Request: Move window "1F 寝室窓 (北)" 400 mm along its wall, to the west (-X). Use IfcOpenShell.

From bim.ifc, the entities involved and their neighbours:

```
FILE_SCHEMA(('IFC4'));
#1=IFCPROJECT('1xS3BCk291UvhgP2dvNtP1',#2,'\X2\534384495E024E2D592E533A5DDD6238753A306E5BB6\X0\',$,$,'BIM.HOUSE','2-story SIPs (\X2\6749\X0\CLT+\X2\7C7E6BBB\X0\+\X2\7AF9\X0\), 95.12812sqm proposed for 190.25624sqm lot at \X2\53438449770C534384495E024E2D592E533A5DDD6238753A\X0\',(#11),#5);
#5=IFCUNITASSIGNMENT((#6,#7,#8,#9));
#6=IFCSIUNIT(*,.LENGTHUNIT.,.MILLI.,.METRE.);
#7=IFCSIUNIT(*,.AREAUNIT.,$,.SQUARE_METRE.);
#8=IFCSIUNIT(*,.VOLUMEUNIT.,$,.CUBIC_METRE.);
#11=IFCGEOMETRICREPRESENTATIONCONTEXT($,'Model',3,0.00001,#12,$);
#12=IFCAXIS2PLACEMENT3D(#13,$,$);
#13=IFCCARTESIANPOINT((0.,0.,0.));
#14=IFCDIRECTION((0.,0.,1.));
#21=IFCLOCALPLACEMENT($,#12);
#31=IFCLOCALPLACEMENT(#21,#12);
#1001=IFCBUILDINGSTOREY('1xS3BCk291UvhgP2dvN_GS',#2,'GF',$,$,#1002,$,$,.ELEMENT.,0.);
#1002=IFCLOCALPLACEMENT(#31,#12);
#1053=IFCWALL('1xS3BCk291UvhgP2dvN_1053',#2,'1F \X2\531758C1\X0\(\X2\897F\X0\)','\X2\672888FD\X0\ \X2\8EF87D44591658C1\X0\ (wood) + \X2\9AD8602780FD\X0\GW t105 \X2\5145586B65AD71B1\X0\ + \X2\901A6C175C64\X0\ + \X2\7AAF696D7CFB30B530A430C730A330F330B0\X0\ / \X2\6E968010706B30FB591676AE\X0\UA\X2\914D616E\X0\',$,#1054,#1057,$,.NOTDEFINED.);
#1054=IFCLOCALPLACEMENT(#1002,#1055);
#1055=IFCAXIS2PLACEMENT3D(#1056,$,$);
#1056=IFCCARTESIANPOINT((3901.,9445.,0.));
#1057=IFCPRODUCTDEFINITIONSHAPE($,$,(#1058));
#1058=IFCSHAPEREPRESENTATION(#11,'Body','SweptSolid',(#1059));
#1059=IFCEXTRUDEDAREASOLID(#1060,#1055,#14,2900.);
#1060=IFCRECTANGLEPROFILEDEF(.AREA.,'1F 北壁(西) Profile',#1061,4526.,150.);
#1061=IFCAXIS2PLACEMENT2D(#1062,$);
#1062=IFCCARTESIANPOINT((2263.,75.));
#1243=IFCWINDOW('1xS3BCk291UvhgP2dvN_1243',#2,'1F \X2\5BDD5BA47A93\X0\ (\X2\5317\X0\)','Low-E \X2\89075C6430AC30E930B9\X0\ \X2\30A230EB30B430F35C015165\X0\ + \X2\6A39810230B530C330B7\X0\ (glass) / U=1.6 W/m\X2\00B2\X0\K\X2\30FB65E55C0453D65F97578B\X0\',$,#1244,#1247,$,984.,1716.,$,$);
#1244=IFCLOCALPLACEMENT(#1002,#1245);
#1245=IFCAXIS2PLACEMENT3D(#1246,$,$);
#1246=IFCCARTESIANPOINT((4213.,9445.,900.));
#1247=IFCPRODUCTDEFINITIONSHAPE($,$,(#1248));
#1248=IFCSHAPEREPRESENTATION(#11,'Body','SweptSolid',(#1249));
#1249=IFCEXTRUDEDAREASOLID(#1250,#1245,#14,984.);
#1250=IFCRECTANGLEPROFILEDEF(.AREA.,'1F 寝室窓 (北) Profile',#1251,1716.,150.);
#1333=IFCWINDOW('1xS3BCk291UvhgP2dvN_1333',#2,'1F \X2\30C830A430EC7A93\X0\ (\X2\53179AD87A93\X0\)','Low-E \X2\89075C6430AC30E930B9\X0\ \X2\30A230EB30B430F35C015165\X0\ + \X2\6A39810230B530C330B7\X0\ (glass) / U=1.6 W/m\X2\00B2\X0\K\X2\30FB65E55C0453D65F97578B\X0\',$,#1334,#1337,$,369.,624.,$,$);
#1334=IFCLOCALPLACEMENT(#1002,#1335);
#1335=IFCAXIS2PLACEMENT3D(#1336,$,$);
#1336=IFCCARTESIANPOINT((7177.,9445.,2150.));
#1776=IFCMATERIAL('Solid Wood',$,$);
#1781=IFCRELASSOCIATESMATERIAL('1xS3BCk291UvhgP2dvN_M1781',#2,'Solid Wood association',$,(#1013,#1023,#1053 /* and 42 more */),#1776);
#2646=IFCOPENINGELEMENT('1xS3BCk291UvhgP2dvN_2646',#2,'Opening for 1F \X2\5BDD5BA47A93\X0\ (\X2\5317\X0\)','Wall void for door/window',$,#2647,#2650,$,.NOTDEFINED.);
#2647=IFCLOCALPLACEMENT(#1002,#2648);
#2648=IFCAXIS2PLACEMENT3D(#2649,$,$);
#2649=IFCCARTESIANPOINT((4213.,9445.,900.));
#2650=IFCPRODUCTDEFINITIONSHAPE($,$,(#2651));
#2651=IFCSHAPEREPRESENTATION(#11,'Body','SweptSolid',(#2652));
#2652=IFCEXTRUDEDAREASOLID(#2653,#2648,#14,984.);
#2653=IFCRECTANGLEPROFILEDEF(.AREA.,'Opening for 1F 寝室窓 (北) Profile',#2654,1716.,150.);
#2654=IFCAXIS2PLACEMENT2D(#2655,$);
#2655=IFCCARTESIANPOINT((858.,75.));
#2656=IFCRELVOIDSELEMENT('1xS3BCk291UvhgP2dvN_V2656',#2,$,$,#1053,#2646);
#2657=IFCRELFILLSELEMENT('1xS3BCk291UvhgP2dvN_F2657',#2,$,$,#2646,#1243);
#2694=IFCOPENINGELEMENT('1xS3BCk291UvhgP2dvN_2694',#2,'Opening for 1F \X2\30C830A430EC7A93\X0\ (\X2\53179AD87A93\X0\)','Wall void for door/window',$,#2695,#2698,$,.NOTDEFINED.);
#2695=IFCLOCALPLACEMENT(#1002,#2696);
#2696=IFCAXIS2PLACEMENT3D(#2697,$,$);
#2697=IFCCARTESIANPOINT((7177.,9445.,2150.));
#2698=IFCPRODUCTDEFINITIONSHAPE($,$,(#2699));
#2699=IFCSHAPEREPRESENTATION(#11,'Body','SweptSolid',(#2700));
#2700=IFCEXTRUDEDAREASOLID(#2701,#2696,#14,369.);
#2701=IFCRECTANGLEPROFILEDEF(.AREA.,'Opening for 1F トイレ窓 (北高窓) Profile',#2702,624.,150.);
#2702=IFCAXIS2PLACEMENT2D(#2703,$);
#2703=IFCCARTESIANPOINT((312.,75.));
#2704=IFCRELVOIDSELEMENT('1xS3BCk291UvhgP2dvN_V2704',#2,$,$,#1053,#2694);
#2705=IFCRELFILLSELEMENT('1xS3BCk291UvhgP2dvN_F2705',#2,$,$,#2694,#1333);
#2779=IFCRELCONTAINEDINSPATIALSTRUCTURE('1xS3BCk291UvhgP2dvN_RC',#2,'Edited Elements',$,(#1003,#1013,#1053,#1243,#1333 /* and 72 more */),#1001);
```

```python
import ifcopenshell
import ifcopenshell.api.geometry
import ifcopenshell.util.placement
import ifcopenshell.util.unit

model = ifcopenshell.open("bim.ifc")
unit_scale = ifcopenshell.util.unit.calculate_unit_scale(model)

window = model.by_id(1243)
opening = window.FillsVoids[0].RelatingOpeningElement
wall = opening.VoidsElements[0].RelatingBuildingElement

wall_matrix = ifcopenshell.util.placement.get_local_placement(wall.ObjectPlacement)
shift = wall_matrix[:3, 0] * -0.4 / unit_scale
before = ifcopenshell.util.placement.get_local_placement(window.ObjectPlacement)[:3, 3].copy()

# The window is not placed relative to its opening, so move both.
for product in (opening, window):
    matrix = ifcopenshell.util.placement.get_local_placement(product.ObjectPlacement)
    matrix[:3, 3] += shift
    ifcopenshell.api.geometry.edit_object_placement(model, product=product, matrix=matrix, is_si=False)

after = ifcopenshell.util.placement.get_local_placement(window.ObjectPlacement)[:3, 3]
print("window moved by", (after - before).round(3) + 0.0)

model.write("bim_updated.ifc")
```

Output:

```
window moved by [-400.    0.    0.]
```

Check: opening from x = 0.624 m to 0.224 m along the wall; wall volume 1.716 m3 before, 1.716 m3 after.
